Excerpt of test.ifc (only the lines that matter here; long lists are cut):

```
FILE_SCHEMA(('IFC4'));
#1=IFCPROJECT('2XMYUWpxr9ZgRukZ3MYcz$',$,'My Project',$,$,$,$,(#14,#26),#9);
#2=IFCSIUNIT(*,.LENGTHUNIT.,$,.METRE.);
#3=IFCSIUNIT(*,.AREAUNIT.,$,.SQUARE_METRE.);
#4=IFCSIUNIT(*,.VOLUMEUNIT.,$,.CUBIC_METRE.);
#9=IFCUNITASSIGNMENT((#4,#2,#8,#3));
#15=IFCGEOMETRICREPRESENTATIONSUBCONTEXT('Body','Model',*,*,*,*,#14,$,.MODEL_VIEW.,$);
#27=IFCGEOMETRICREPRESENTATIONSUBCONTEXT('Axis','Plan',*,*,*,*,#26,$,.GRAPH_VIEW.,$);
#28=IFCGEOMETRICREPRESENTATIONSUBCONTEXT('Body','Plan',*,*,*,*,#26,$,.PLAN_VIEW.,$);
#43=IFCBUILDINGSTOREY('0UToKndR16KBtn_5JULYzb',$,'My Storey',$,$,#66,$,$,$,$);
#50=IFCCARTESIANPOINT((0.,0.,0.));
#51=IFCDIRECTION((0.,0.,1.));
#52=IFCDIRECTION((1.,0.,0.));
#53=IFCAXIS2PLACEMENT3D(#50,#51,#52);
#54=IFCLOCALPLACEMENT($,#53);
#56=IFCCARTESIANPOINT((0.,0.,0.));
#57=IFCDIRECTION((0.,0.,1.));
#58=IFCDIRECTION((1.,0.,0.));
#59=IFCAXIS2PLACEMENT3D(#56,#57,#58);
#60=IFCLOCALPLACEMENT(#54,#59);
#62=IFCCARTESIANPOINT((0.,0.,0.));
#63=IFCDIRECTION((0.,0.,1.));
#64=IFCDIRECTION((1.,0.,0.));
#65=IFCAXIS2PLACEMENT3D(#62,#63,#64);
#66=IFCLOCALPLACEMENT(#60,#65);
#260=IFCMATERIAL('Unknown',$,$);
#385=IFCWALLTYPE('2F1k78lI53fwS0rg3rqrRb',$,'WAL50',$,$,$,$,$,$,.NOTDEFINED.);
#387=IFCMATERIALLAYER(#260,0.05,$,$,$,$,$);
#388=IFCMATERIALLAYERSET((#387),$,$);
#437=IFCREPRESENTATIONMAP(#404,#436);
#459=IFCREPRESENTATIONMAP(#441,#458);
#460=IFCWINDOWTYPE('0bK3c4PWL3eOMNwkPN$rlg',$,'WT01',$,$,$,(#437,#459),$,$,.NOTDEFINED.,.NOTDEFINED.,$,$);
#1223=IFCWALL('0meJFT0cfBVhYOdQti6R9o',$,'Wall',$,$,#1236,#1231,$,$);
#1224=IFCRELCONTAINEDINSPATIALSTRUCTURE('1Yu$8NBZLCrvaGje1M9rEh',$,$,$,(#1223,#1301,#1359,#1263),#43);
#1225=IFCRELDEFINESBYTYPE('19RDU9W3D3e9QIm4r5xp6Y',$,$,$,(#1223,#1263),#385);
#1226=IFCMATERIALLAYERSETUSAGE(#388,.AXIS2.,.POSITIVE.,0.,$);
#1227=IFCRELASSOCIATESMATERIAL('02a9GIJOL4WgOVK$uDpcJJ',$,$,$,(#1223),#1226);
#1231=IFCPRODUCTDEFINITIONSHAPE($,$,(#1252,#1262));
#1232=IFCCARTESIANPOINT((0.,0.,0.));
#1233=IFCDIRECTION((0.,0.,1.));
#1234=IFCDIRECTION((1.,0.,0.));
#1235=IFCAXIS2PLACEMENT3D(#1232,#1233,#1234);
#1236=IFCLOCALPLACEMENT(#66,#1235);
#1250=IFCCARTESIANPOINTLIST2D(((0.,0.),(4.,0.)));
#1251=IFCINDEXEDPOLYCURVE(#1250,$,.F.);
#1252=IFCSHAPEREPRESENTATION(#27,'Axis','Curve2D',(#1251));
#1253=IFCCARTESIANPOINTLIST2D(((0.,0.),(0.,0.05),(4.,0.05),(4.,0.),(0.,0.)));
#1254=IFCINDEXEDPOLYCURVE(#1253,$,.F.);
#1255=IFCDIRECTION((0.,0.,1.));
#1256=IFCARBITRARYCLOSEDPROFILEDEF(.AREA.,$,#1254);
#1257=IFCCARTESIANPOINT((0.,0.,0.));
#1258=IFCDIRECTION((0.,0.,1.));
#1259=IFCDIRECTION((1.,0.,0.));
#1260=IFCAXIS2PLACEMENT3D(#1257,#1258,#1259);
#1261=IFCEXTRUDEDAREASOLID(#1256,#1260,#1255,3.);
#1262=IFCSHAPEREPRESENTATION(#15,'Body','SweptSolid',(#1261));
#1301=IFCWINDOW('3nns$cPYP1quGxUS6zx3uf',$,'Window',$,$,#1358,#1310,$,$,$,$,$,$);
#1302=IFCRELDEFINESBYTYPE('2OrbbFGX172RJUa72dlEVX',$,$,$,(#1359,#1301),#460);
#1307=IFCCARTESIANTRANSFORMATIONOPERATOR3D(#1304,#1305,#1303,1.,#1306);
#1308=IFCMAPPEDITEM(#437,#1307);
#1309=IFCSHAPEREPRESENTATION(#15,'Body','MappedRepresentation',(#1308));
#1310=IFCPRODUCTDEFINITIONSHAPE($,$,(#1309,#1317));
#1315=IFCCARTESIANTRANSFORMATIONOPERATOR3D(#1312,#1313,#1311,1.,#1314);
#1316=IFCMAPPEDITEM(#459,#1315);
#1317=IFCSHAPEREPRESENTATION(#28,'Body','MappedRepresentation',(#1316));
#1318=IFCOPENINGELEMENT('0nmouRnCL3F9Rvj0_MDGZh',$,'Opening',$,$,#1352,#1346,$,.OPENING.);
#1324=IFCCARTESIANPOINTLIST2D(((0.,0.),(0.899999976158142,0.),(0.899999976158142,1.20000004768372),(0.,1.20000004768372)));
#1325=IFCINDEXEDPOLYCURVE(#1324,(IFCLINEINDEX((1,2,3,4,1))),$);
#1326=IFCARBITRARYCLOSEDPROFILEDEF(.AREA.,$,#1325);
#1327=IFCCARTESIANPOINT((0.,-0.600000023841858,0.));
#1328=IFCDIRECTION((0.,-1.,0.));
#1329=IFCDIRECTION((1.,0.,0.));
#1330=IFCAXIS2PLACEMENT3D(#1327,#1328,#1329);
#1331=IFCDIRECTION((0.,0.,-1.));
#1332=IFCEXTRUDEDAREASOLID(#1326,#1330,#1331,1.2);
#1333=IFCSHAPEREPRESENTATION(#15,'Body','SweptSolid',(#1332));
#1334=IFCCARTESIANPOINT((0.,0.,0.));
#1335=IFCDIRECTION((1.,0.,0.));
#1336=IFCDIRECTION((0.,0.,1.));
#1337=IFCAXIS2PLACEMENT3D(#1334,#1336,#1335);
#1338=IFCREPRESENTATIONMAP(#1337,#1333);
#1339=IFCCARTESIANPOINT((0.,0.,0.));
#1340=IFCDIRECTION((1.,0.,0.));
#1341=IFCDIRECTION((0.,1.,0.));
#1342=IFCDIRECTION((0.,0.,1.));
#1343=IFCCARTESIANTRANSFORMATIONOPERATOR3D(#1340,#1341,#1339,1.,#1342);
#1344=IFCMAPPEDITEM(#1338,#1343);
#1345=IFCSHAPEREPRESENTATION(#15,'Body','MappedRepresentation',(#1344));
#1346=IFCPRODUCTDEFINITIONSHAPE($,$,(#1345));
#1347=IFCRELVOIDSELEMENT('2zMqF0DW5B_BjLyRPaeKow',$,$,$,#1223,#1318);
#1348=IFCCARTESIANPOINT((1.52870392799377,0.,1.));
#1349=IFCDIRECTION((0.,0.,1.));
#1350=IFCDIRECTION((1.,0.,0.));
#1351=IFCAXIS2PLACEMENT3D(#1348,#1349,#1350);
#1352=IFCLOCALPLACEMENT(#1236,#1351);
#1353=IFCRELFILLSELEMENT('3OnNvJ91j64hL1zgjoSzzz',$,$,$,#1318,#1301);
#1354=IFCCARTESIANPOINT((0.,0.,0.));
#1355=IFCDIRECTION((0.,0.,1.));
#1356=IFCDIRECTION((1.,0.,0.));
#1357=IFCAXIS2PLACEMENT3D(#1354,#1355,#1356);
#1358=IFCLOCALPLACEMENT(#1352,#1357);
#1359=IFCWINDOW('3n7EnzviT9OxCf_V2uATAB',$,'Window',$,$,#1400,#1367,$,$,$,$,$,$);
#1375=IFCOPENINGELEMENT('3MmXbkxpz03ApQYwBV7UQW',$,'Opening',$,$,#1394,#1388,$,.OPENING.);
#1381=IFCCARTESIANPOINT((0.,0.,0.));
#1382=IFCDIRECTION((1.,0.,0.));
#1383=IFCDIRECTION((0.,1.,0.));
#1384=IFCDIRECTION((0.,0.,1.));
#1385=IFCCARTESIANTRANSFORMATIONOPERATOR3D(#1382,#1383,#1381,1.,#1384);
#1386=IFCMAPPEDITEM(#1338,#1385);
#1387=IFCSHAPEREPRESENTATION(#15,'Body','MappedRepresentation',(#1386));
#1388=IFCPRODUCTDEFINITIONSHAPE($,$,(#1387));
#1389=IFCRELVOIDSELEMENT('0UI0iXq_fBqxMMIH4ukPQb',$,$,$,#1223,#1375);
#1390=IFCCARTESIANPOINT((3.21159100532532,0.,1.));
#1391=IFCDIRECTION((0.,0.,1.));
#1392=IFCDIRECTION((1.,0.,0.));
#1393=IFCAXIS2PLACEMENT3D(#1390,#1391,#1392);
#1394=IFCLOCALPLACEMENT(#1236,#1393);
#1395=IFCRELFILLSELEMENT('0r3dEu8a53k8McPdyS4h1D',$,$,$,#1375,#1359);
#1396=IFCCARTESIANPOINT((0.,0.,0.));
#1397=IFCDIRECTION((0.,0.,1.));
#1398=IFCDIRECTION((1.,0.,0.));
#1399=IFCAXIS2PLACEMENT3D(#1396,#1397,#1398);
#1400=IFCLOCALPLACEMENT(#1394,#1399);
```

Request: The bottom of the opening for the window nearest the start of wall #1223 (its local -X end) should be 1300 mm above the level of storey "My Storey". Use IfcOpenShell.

```python
import numpy as np
import ifcopenshell
import ifcopenshell.api.geometry
import ifcopenshell.geom
import ifcopenshell.util.element
import ifcopenshell.util.placement
import ifcopenshell.util.shape
import ifcopenshell.util.unit

model = ifcopenshell.open("test.ifc")
unit_scale = ifcopenshell.util.unit.calculate_unit_scale(model)

window = model.by_guid("3nns$cPYP1quGxUS6zx3uf")
opening = window.FillsVoids[0].RelatingOpeningElement
storey = ifcopenshell.util.element.get_container(window, ifc_class="IfcBuildingStorey")
level = ifcopenshell.util.placement.get_local_placement(storey.ObjectPlacement)[2, 3]

# The opening's origin need not be at the sill, so measure its lowest point.
shape = ifcopenshell.geom.create_shape(ifcopenshell.geom.settings(), opening)
bottom = ifcopenshell.util.shape.get_shape_bottom_elevation(shape, shape.geometry) / unit_scale
dz = level + 1.3 - bottom

shift = np.array([0.0, 0.0, dz])
# The window is placed relative to its opening, so it follows when the opening moves.
matrix = ifcopenshell.util.placement.get_local_placement(opening.ObjectPlacement)
matrix[:3, 3] += shift
ifcopenshell.api.geometry.edit_object_placement(
    model, product=opening, matrix=matrix, is_si=False, should_transform_children=True
)

print(f"moved by {dz * unit_scale:+.3f} m")

model.write("test_v2.ifc")
```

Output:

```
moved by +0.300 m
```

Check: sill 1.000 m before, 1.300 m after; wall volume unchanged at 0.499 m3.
